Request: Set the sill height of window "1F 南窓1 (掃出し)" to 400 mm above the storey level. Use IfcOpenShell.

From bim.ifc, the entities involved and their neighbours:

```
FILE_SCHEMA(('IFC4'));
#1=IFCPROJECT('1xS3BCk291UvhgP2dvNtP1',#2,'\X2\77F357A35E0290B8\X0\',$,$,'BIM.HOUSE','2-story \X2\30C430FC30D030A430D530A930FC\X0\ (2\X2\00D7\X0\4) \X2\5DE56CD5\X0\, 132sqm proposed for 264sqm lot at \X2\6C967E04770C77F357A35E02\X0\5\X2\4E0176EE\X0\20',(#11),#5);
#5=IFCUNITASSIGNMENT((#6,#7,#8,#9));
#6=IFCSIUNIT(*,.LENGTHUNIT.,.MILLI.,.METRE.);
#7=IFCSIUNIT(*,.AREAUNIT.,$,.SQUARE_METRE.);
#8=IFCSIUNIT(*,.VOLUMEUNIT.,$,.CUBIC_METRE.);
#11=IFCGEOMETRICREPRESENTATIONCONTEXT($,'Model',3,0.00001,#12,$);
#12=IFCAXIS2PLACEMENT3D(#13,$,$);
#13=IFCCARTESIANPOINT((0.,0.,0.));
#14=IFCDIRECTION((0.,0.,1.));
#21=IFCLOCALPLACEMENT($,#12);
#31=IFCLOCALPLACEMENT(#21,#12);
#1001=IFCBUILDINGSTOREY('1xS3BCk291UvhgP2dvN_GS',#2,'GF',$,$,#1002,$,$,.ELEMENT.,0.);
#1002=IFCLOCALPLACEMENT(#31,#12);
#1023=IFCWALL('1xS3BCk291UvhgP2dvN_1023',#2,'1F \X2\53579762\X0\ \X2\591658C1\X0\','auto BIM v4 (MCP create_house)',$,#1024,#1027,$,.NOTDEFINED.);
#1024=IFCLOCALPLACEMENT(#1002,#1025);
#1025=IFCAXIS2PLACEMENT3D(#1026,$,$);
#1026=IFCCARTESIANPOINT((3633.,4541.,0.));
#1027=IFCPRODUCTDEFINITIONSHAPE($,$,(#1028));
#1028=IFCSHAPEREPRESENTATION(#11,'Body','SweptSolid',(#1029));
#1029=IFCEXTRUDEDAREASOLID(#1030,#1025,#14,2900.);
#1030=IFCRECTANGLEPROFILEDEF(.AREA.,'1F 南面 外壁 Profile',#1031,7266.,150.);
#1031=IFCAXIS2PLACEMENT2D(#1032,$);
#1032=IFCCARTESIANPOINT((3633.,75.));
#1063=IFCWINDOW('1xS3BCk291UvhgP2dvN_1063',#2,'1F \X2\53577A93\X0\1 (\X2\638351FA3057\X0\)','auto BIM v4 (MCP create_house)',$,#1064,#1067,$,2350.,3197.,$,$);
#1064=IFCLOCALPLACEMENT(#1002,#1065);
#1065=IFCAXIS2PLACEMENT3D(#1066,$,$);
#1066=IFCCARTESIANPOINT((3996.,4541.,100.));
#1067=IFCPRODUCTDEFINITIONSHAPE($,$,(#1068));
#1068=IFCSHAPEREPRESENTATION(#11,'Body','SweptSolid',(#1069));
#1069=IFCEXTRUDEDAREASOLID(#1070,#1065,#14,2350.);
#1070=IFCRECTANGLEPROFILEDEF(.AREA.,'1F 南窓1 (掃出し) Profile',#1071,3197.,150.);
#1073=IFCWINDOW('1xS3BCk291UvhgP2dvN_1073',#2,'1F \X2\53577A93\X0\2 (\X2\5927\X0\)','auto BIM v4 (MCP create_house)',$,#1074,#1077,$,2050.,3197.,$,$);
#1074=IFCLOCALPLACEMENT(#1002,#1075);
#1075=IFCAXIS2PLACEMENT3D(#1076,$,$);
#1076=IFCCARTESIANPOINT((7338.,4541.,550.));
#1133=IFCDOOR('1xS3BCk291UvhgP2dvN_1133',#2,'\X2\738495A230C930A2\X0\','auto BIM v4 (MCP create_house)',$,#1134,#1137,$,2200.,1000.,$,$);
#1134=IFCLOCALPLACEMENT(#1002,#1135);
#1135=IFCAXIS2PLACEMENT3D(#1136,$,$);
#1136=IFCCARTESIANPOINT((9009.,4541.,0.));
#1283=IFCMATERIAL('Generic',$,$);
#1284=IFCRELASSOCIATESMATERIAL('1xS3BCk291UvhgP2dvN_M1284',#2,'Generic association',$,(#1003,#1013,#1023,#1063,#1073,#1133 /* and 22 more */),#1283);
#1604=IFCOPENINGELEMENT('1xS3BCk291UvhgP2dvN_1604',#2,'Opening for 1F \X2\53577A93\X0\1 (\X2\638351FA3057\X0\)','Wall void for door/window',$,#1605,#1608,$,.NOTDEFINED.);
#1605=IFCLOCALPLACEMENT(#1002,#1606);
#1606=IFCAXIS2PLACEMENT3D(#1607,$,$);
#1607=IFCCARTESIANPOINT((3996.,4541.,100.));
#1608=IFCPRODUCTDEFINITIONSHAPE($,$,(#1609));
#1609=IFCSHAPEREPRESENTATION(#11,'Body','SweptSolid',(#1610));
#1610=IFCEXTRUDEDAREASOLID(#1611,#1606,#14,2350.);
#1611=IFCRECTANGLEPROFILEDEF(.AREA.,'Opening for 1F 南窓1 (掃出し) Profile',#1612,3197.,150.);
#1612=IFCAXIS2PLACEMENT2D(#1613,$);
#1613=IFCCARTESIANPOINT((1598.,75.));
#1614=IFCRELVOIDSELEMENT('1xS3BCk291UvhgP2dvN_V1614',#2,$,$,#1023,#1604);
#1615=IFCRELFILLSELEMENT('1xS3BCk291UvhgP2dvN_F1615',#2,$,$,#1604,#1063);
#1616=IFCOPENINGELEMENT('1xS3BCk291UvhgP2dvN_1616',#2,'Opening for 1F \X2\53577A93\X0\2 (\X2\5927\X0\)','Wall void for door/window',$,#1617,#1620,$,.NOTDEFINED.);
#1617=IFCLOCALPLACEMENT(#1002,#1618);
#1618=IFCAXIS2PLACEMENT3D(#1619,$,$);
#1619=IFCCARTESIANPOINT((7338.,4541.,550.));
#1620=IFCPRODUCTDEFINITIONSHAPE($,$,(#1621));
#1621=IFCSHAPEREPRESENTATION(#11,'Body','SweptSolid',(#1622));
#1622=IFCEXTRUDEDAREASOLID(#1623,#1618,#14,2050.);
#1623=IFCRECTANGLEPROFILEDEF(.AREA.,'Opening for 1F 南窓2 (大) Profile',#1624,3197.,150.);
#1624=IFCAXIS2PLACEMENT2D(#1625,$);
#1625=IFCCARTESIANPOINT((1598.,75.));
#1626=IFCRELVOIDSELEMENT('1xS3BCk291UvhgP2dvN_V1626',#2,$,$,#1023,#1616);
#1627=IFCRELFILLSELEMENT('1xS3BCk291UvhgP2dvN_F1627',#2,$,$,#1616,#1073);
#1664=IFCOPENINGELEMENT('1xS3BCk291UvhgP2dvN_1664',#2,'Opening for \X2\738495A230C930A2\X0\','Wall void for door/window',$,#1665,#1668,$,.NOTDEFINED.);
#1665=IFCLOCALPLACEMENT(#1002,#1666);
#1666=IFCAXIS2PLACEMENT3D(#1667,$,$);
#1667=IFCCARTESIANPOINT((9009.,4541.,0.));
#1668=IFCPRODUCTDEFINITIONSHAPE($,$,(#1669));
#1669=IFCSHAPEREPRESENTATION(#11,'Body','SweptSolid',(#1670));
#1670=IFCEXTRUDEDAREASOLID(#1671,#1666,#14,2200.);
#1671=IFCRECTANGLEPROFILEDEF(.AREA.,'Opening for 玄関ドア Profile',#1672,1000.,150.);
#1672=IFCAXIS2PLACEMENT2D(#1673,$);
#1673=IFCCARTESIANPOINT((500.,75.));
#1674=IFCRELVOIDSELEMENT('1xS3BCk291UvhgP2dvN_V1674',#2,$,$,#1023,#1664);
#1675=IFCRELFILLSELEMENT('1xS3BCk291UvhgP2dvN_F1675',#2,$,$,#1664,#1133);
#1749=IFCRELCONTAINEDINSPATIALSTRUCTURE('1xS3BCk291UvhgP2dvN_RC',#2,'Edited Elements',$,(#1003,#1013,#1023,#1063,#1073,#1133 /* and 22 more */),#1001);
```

```python
import numpy as np
import ifcopenshell
import ifcopenshell.api.geometry
import ifcopenshell.geom
import ifcopenshell.util.element
import ifcopenshell.util.placement
import ifcopenshell.util.shape
import ifcopenshell.util.unit

model = ifcopenshell.open("bim.ifc")
unit_scale = ifcopenshell.util.unit.calculate_unit_scale(model)

window = model.by_guid("1xS3BCk291UvhgP2dvN_1063")
opening = window.FillsVoids[0].RelatingOpeningElement
storey = ifcopenshell.util.element.get_container(window, ifc_class="IfcBuildingStorey")
level = ifcopenshell.util.placement.get_local_placement(storey.ObjectPlacement)[2, 3]

# The opening's origin need not be at the sill, so measure its lowest point.
shape = ifcopenshell.geom.create_shape(ifcopenshell.geom.settings(), opening)
bottom = ifcopenshell.util.shape.get_shape_bottom_elevation(shape, shape.geometry) / unit_scale
dz = level + 400.0 - bottom

shift = np.array([0.0, 0.0, dz])
# The window is not placed relative to its opening, so move both.
for product in (opening, window):
    matrix = ifcopenshell.util.placement.get_local_placement(product.ObjectPlacement)
    matrix[:3, 3] += shift
    ifcopenshell.api.geometry.edit_object_placement(model, product=product, matrix=matrix, is_si=False)

print(f"moved by {dz * unit_scale:+.3f} m")

model.write("bim_rev.ifc")
```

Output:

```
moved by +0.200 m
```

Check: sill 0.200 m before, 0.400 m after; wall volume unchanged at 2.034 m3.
